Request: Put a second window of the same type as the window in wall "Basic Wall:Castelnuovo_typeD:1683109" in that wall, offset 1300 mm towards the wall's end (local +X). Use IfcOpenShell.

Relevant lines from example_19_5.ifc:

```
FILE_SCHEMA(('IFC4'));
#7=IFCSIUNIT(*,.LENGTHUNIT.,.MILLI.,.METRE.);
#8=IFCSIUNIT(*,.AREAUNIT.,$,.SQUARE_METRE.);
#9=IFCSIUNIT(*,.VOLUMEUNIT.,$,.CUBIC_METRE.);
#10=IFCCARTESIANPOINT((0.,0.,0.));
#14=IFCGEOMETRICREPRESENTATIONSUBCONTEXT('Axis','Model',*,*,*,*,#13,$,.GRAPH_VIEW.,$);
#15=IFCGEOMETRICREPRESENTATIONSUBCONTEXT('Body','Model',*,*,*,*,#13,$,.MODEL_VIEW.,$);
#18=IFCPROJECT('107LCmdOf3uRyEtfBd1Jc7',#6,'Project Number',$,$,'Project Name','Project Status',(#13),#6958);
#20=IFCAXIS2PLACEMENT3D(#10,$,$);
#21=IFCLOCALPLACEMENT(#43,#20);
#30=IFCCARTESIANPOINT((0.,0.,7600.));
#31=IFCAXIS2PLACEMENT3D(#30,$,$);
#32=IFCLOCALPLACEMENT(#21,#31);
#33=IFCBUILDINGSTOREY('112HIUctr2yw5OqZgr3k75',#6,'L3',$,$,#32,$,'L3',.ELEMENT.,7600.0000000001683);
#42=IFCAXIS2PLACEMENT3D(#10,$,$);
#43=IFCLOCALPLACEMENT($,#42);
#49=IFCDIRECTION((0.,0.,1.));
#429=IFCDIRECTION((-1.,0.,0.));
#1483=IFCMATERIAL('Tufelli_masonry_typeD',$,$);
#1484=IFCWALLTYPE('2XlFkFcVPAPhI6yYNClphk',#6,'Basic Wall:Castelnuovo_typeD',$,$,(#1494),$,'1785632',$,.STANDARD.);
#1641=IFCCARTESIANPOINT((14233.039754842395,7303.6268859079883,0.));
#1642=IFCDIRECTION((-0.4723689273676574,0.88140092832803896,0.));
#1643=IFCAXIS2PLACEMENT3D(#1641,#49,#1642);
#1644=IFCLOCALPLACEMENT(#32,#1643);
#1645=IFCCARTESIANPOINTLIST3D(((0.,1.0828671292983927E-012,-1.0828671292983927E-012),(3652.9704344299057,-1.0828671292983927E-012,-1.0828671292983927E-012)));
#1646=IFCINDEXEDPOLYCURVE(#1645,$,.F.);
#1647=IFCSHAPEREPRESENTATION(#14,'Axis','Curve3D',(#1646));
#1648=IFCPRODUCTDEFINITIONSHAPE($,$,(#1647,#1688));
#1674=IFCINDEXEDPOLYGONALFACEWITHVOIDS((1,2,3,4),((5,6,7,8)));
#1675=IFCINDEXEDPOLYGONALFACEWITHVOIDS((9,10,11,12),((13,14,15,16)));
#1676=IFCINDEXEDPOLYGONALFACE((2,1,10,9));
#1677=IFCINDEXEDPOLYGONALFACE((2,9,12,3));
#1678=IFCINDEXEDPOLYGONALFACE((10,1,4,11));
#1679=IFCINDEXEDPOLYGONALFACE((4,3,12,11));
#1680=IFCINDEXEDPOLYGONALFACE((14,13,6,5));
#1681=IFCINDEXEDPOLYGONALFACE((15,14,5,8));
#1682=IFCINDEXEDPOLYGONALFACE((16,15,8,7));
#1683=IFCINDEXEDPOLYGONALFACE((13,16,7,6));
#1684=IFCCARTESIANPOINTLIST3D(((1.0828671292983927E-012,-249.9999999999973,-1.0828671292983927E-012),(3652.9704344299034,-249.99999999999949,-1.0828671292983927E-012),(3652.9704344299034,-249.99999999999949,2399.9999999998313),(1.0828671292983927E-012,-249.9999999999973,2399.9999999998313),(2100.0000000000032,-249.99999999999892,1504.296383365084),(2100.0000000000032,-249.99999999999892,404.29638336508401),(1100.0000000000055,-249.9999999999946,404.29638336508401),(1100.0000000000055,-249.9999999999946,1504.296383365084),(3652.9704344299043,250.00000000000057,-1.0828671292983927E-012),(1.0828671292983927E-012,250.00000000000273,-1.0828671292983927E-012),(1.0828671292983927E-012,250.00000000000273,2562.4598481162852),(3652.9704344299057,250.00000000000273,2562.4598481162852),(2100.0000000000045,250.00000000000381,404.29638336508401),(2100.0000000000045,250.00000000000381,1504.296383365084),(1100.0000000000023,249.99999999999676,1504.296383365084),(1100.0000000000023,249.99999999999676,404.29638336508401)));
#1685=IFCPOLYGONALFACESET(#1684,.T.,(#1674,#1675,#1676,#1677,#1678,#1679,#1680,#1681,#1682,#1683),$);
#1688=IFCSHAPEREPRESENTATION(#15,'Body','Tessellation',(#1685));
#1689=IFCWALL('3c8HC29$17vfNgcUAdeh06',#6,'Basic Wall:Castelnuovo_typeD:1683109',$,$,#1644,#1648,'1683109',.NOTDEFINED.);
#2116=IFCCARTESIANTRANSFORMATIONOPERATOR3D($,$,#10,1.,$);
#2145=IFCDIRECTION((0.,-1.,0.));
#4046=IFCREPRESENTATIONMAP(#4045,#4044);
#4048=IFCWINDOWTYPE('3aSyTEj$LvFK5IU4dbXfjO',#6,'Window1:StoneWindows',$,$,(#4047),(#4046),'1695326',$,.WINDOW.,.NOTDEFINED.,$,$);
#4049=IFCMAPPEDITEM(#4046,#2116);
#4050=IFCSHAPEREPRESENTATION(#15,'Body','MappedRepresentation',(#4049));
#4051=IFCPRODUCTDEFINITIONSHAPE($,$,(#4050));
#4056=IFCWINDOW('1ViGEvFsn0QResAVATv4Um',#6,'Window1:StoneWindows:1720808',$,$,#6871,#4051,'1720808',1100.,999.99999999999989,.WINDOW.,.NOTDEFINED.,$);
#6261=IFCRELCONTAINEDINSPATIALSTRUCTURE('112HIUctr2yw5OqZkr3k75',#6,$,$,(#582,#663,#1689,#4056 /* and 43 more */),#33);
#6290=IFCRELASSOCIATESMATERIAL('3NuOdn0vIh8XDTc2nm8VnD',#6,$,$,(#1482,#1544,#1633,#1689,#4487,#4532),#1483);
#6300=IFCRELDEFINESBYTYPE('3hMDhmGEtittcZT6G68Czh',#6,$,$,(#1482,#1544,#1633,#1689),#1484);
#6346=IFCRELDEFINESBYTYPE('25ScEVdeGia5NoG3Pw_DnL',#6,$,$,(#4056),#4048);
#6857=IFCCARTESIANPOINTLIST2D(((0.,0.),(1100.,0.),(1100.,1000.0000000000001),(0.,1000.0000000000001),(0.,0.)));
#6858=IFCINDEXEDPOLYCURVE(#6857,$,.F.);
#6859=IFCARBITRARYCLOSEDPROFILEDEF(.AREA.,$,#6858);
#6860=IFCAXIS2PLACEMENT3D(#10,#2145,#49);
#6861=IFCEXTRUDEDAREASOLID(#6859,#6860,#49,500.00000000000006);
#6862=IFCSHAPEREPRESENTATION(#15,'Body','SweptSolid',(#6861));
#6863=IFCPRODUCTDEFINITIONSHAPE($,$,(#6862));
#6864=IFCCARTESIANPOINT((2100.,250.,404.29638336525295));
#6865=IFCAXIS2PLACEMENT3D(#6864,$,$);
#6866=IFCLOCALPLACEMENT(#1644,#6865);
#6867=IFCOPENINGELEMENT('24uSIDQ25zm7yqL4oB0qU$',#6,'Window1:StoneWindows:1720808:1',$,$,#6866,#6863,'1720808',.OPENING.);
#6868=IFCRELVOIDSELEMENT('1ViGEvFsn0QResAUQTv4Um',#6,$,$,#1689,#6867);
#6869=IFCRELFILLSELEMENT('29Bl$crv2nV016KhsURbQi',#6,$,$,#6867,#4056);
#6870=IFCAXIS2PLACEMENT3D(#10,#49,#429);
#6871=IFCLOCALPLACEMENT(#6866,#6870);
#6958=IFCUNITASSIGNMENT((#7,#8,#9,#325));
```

```python
import ifcopenshell
import ifcopenshell.api.feature
import ifcopenshell.api.geometry
import ifcopenshell.api.root
import ifcopenshell.geom
import ifcopenshell.util.element
import ifcopenshell.util.placement
import ifcopenshell.util.shape

model = ifcopenshell.open("example_19_5.ifc")
settings = ifcopenshell.geom.settings()


def volume(element):
    """Net volume in cubic metres, openings subtracted."""
    shape = ifcopenshell.geom.create_shape(settings, element)
    return ifcopenshell.util.shape.get_volume(shape.geometry)


def reuse_history(source, copy):
    """copy_class also copies each property set's owner history, people and application; keep the originals."""
    for rel in copy.IsDefinedBy:
        if rel.is_a("IfcRelDefinesByProperties") and (history := rel.RelatingPropertyDefinition.OwnerHistory):
            rel.RelatingPropertyDefinition.OwnerHistory = source.OwnerHistory
            ifcopenshell.util.element.remove_deep2(model, history)


window = model.by_id(4056)
opening = window.FillsVoids[0].RelatingOpeningElement
wall = opening.VoidsElements[0].RelatingBuildingElement
before = volume(wall)
shift = ifcopenshell.util.placement.get_local_placement(wall.ObjectPlacement)[:3, 0] * 1300.0

# copy_class copies the void relationship, type, container and properties, but no geometry.
new_opening = ifcopenshell.api.root.copy_class(model, product=opening)
new_opening.Representation = ifcopenshell.util.element.copy_deep(
    model, opening.Representation, exclude=["IfcGeometricRepresentationContext", "IfcRepresentationMap"]
)
new_opening.Name = "Window1:StoneWindows"
new_opening.Tag = None
new_window = ifcopenshell.api.root.copy_class(model, product=window)
new_window.Representation = ifcopenshell.util.element.copy_deep(
    model, window.Representation, exclude=["IfcGeometricRepresentationContext", "IfcRepresentationMap"]
)
new_window.Name = "Window1:StoneWindows"
new_window.Tag = None
reuse_history(window, new_window)
ifcopenshell.api.feature.add_filling(model, opening=new_opening, element=new_window)

for old, new in ((opening, new_opening), (window, new_window)):
    matrix = ifcopenshell.util.placement.get_local_placement(old.ObjectPlacement)
    matrix[:3, 3] += shift
    ifcopenshell.api.geometry.edit_object_placement(model, product=new, matrix=matrix, is_si=False)

after = volume(wall)

print(f"wall volume {before:.3f} -> {after:.3f} m3")

model.write("example_19_5-out.ifc")
```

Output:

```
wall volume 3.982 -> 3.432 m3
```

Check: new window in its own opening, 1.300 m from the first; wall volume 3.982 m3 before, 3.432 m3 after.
